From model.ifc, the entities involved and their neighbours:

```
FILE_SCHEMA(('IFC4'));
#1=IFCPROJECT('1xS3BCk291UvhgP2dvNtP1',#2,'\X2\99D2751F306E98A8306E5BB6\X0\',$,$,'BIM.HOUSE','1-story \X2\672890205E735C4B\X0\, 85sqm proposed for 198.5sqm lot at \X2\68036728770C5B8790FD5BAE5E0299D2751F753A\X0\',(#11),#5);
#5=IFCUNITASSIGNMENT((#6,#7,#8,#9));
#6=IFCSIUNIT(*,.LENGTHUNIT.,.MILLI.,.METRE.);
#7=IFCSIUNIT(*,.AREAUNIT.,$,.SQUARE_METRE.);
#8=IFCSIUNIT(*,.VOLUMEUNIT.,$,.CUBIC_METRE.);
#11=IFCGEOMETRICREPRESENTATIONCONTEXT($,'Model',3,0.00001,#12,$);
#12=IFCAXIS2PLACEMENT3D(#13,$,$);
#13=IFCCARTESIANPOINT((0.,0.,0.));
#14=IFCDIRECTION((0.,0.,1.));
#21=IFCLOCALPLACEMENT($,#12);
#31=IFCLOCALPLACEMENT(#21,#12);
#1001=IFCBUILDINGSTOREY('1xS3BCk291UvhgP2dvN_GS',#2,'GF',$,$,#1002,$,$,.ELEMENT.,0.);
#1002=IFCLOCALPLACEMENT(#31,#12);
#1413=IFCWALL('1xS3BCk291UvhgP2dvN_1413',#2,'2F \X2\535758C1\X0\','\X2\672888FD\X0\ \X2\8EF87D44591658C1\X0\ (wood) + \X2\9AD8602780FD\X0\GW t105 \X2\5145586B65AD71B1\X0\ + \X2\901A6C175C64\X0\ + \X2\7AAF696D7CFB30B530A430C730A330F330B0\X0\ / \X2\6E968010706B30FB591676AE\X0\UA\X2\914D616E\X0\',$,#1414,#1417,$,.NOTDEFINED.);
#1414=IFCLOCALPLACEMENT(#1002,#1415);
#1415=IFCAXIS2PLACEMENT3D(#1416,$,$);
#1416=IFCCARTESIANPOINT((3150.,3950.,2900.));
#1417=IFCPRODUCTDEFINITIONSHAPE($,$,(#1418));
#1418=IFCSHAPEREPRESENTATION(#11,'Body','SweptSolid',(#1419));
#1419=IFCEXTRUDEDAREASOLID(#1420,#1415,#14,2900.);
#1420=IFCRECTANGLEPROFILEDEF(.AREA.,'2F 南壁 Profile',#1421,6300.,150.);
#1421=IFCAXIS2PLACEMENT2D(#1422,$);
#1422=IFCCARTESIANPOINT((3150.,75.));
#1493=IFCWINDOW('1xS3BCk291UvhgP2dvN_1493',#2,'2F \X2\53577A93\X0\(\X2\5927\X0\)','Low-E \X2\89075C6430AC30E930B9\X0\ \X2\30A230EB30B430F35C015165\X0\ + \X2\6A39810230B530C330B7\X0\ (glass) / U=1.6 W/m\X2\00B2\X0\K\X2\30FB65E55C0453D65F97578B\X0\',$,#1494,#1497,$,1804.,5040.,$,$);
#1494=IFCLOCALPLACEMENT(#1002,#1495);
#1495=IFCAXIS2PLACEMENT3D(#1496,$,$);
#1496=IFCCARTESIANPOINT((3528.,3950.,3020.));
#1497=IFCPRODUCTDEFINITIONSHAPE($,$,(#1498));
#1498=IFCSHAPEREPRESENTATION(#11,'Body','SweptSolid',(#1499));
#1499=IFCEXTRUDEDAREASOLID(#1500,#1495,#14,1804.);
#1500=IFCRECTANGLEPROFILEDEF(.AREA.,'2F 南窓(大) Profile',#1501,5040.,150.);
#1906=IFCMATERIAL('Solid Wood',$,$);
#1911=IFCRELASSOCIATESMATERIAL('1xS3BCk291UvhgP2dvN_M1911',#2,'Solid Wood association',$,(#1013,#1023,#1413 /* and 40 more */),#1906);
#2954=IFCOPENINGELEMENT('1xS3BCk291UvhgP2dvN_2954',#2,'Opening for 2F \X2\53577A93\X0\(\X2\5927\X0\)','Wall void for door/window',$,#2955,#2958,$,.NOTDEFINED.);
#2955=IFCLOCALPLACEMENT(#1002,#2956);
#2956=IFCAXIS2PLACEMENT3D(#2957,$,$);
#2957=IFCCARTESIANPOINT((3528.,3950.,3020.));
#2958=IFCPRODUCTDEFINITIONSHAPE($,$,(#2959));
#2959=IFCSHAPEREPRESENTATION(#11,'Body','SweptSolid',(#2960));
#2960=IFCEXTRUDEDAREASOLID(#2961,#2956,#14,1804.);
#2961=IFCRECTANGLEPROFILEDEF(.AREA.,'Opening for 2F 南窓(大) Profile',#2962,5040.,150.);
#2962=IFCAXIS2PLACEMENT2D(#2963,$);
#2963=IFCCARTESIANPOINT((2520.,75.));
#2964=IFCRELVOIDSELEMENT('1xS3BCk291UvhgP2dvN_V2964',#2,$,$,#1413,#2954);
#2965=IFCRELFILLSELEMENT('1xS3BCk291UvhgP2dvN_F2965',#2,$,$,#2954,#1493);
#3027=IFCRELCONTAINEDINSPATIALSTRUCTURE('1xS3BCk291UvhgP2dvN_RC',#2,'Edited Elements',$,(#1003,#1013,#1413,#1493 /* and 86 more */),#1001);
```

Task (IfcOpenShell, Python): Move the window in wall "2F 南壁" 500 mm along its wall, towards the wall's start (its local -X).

```python
import ifcopenshell
import ifcopenshell.api.geometry
import ifcopenshell.util.placement

model = ifcopenshell.open("model.ifc")

window = model.by_guid("1xS3BCk291UvhgP2dvN_1493")
opening = window.FillsVoids[0].RelatingOpeningElement
wall = opening.VoidsElements[0].RelatingBuildingElement

wall_matrix = ifcopenshell.util.placement.get_local_placement(wall.ObjectPlacement)
shift = wall_matrix[:3, 0] * -500.0
before = ifcopenshell.util.placement.get_local_placement(window.ObjectPlacement)[:3, 3].copy()

# The window is not placed relative to its opening, so move both.
for product in (opening, window):
    matrix = ifcopenshell.util.placement.get_local_placement(product.ObjectPlacement)
    matrix[:3, 3] += shift
    ifcopenshell.api.geometry.edit_object_placement(model, product=product, matrix=matrix, is_si=False)

after = ifcopenshell.util.placement.get_local_placement(window.ObjectPlacement)[:3, 3]
print("window moved by", (after - before).round(3) + 0.0)

model.write("model-out.ifc")
```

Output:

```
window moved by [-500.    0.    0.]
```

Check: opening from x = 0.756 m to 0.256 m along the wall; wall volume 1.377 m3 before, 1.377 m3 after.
